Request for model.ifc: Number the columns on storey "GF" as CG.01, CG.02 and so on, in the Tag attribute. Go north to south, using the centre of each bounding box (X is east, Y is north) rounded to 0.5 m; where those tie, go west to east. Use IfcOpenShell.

First a look at what the model holds.

```python
import ifcopenshell
import ifcopenshell.util.element
import ifcopenshell.util.placement

model = ifcopenshell.open("model.ifc")
print(model.schema)
storey = next(s for s in model.by_type("IfcBuildingStorey") if s.Name == "GF")
columns = [e for e in ifcopenshell.util.element.get_decomposition(storey) if e.is_a("IfcColumn")]
for e in sorted(columns, key=lambda e: e.id()):
    origin = ifcopenshell.util.placement.get_local_placement(e.ObjectPlacement)[:3, 3]
    print(e.id(), e.Tag, e.Name, origin.round(2) + 0.0, sep=" | ")
```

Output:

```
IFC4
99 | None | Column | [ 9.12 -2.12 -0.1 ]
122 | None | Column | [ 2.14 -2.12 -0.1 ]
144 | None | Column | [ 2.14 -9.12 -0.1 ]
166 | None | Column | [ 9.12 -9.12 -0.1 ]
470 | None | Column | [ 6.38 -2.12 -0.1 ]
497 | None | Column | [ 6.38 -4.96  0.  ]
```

```python
import ifcopenshell
import ifcopenshell.geom
import ifcopenshell.util.element
import ifcopenshell.util.shape

model = ifcopenshell.open("model.ifc")
settings = ifcopenshell.geom.settings()
settings.set("use-world-coords", True)


def centre(element):
    shape = ifcopenshell.geom.create_shape(settings, element)
    return ifcopenshell.util.shape.get_bbox_centroid(shape.geometry)


storey = next(s for s in model.by_type("IfcBuildingStorey") if s.Name == "GF")
columns = [e for e in ifcopenshell.util.element.get_decomposition(storey) if e.is_a("IfcColumn")]

# Insertion points can sit at a corner or the storey origin, so sort by the geometry (in metres).
centres = {e: centre(e) for e in columns}
columns.sort(key=lambda e: (-round(centres[e][1] / 0.5), centres[e][0]))

for i, e in enumerate(columns, start=1):
    number = f"CG.{i:02d}"
    e.Tag = number
    print(e.id(), number)

model.write("model_v2.ifc")
```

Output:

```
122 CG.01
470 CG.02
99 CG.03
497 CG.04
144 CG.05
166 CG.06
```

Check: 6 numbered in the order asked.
